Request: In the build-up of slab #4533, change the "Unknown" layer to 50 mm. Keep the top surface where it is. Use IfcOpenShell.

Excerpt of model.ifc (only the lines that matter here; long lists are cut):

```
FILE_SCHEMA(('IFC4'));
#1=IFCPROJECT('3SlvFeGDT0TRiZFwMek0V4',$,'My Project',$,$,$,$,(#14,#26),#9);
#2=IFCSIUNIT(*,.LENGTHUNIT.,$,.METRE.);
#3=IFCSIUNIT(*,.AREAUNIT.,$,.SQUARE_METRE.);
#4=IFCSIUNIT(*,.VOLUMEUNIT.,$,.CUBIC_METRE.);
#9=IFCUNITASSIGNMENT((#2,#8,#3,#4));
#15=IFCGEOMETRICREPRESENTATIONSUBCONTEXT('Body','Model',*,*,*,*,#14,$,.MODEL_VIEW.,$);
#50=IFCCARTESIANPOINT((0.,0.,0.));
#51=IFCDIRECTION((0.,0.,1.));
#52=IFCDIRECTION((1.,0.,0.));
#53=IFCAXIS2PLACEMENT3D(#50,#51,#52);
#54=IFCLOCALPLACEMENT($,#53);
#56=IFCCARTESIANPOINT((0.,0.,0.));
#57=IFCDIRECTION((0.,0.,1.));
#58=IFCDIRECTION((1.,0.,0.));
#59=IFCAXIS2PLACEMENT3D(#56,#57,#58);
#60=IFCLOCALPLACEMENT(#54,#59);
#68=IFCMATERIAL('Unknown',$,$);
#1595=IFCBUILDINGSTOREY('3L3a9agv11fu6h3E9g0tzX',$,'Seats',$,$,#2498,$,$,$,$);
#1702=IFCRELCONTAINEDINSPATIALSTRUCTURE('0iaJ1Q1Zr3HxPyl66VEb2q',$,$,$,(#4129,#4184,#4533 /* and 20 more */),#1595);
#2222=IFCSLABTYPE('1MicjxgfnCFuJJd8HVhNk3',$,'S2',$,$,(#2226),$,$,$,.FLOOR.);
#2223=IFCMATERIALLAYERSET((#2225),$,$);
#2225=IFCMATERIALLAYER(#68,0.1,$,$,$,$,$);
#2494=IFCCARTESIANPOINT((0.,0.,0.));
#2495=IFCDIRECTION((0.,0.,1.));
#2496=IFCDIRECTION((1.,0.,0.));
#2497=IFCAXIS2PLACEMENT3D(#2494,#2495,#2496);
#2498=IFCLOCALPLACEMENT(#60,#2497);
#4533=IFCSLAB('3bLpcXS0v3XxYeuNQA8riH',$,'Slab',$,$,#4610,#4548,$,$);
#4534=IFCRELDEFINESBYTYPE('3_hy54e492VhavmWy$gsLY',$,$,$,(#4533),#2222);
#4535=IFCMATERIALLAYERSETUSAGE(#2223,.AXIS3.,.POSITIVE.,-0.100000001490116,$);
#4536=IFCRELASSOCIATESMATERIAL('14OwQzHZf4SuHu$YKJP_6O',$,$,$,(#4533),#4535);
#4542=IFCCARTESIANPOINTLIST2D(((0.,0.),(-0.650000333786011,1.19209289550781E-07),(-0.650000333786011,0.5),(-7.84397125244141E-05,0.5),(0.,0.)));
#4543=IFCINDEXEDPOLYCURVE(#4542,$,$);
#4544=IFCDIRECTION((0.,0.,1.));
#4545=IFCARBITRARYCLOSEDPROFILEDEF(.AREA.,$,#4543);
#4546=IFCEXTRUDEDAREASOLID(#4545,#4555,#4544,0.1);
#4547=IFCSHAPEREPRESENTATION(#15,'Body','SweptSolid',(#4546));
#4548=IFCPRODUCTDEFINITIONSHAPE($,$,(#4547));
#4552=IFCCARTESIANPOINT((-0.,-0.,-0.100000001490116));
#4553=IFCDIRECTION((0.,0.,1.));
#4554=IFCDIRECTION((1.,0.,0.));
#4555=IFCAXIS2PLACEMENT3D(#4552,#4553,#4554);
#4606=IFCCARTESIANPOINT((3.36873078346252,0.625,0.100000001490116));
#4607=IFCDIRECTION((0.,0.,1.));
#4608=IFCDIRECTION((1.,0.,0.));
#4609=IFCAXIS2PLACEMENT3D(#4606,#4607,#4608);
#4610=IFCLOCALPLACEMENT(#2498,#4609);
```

```python
import ifcopenshell
import ifcopenshell.util.element
import ifcopenshell.util.representation
import ifcopenshell.util.unit

model = ifcopenshell.open("model.ifc")
unit_scale = ifcopenshell.util.unit.calculate_unit_scale(model)

layer_set = model.by_id(2223)
layer = next(l for l in layer_set.MaterialLayers if l.Material and l.Material.Name == "Unknown")
change = 0.05 / unit_scale - layer.LayerThickness
layer.LayerThickness += change

# Geometry does not follow the layer set by itself.
slabs = [e for e in ifcopenshell.util.element.get_elements_by_material(model, layer_set) if e.is_a("IfcSlab")]
for slab in sorted(slabs, key=lambda e: e.id()):
    body = ifcopenshell.util.representation.get_representation(slab, "Model", "Body")
    solid = body.Items[0]
    old_depth = solid.Depth
    solid.Depth += change
    # Extruded upwards: lower the start of the extrusion so the top stays.
    x, y, z = solid.Position.Location.Coordinates
    solid.Position.Location = model.createIfcCartesianPoint((x, y, z - change))
    print(slab.id(), f"{old_depth:g} -> {solid.Depth:g}")

# The layers are counted up from the underside, which has moved.
for usage in {ifcopenshell.util.element.get_material(slab) for slab in slabs}:
    usage.OffsetFromReferenceLine -= change

model.write("model_edited.ifc")
```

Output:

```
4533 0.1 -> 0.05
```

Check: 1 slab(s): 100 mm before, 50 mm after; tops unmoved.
